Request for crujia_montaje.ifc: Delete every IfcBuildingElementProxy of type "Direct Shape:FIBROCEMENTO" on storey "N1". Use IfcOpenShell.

First a look at what the model holds.

```python
import ifcopenshell
import ifcopenshell.util.element

model = ifcopenshell.open("crujia_montaje.ifc")
print(model.schema)
storey = next(s for s in model.by_type("IfcBuildingStorey") if s.Name == "N1")
proxies = [e for e in ifcopenshell.util.element.get_decomposition(storey) if e.is_a("IfcBuildingElementProxy")]
seen = {}
for e in proxies:
    element_type = ifcopenshell.util.element.get_type(e)
    name = element_type.Name if element_type not in (None, e) else None
    seen[name] = seen.get(name, 0) + 1
for name, count in sorted(seen.items(), key=str):
    print(count, "x", name)
```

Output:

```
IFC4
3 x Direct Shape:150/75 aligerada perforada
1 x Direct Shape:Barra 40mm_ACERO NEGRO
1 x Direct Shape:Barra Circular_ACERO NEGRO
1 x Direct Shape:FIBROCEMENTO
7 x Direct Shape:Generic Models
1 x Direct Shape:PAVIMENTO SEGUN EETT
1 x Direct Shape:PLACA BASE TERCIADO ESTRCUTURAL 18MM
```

```python
import ifcopenshell
import ifcopenshell.api.root
import ifcopenshell.util.element

model = ifcopenshell.open("crujia_montaje.ifc")

storey = next(s for s in model.by_type("IfcBuildingStorey") if s.Name == "N1")
proxies = [e for e in ifcopenshell.util.element.get_decomposition(storey) if e.is_a("IfcBuildingElementProxy")]
targets = [e for e in proxies if (t := ifcopenshell.util.element.get_type(e)) not in (None, e) and t.Name == "Direct Shape:FIBROCEMENTO"]

for e in targets:
    ifcopenshell.api.root.remove_product(model, product=e)
print(len(targets), "removed")

model.write("crujia_montaje_updated.ifc")
```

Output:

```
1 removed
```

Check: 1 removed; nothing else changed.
